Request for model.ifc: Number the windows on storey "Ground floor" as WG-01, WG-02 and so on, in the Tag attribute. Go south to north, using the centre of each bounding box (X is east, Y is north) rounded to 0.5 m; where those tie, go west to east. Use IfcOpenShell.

First a look at what the model holds.

```python
import ifcopenshell
import ifcopenshell.util.element
import ifcopenshell.util.placement

model = ifcopenshell.open("model.ifc")
print(model.schema)
storey = next(s for s in model.by_type("IfcBuildingStorey") if s.Name == "Ground floor")
windows = [e for e in ifcopenshell.util.element.get_decomposition(storey) if e.is_a("IfcWindow")]
for e in sorted(windows, key=lambda e: e.id()):
    origin = ifcopenshell.util.placement.get_local_placement(e.ObjectPlacement)[:3, 3]
    print(e.id(), e.Tag, e.Name, origin.round(2) + 0.0, sep=" | ")
```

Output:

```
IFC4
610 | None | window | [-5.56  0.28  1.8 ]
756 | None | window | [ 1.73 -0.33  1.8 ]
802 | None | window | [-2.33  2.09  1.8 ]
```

```python
import ifcopenshell
import ifcopenshell.geom
import ifcopenshell.util.element
import ifcopenshell.util.shape

model = ifcopenshell.open("model.ifc")
settings = ifcopenshell.geom.settings()
settings.set("use-world-coords", True)


def centre(element):
    shape = ifcopenshell.geom.create_shape(settings, element)
    return ifcopenshell.util.shape.get_bbox_centroid(shape.geometry)


storey = next(s for s in model.by_type("IfcBuildingStorey") if s.Name == "Ground floor")
windows = [e for e in ifcopenshell.util.element.get_decomposition(storey) if e.is_a("IfcWindow")]

# Insertion points can sit at a corner or the storey origin, so sort by the geometry (in metres).
centres = {e: centre(e) for e in windows}
windows.sort(key=lambda e: (round(centres[e][1] / 0.5), centres[e][0]))

for i, e in enumerate(windows, start=1):
    number = f"WG-{i:02d}"
    e.Tag = number
    print(e.id(), number)

model.write("model_updated.ifc")
```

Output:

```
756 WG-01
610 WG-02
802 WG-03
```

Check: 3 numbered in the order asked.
